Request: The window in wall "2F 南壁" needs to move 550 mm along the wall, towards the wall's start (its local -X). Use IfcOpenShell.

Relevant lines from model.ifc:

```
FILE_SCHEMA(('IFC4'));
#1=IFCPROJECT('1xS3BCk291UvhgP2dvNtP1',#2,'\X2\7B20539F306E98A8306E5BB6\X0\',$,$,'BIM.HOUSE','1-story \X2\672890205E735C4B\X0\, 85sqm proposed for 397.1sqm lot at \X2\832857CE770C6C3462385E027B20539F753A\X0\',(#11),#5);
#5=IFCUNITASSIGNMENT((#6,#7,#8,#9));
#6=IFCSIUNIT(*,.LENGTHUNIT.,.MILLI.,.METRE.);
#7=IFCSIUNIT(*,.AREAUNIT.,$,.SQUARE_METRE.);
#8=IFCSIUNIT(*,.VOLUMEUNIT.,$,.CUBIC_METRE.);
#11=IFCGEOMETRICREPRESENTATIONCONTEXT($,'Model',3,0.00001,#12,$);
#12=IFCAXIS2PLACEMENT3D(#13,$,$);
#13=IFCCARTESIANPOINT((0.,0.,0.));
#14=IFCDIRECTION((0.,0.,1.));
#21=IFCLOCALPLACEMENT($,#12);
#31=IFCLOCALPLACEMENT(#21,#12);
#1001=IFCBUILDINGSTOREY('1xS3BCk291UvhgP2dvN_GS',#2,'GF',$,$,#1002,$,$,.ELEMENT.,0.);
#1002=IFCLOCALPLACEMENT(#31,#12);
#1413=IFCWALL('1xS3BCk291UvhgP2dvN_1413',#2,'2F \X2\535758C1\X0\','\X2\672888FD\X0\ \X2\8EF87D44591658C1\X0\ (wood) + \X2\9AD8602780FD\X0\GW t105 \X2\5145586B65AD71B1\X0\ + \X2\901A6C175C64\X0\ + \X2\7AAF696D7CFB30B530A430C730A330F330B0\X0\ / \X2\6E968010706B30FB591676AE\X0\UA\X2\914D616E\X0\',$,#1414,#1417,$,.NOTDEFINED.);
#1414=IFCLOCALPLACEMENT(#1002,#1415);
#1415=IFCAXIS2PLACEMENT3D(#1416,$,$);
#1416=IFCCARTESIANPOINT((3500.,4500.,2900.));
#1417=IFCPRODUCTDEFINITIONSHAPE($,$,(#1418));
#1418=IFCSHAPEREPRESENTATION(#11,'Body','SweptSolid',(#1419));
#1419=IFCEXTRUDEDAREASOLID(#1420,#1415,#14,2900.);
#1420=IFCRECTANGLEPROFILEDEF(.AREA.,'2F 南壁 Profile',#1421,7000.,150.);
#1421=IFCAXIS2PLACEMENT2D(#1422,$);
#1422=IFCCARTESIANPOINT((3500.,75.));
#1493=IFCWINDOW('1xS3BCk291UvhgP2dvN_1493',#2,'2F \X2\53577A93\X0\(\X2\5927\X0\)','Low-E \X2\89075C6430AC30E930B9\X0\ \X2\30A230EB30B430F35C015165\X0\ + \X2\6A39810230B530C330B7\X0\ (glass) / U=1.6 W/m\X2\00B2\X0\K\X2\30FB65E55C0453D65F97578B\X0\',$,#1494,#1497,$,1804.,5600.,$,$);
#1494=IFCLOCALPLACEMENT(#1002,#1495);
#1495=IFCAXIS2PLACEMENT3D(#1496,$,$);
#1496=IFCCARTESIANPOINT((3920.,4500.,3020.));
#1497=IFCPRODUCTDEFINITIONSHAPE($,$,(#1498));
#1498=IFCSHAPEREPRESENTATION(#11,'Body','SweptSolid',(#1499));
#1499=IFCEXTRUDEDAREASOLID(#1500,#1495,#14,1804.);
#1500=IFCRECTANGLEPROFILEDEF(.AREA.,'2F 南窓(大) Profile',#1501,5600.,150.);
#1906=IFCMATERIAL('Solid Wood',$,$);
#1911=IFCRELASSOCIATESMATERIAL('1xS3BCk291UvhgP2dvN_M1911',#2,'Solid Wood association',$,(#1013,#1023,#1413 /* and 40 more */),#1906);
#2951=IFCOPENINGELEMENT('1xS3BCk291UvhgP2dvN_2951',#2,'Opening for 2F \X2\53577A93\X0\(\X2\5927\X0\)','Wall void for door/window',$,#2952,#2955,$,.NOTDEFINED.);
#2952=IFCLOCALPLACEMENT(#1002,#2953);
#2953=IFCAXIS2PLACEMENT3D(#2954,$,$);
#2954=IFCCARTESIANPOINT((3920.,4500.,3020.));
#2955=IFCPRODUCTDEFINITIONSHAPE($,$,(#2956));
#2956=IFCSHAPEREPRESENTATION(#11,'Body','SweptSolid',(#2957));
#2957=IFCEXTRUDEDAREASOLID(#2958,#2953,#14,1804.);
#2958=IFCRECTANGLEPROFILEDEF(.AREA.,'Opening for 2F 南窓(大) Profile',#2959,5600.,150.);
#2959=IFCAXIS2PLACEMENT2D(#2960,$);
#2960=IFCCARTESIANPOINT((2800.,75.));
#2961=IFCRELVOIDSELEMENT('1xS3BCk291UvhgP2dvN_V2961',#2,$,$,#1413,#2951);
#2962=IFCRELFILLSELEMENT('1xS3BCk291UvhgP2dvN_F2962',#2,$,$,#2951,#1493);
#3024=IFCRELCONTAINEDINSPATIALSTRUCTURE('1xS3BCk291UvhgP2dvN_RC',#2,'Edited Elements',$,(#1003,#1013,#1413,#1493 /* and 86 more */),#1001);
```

```python
import ifcopenshell
import ifcopenshell.api.geometry
import ifcopenshell.util.placement

model = ifcopenshell.open("model.ifc")

window = model.by_guid("1xS3BCk291UvhgP2dvN_1493")
opening = window.FillsVoids[0].RelatingOpeningElement
wall = opening.VoidsElements[0].RelatingBuildingElement

wall_matrix = ifcopenshell.util.placement.get_local_placement(wall.ObjectPlacement)
shift = wall_matrix[:3, 0] * -550.0
before = ifcopenshell.util.placement.get_local_placement(window.ObjectPlacement)[:3, 3].copy()

# The window is not placed relative to its opening, so move both.
for product in (opening, window):
    matrix = ifcopenshell.util.placement.get_local_placement(product.ObjectPlacement)
    matrix[:3, 3] += shift
    ifcopenshell.api.geometry.edit_object_placement(model, product=product, matrix=matrix, is_si=False)

after = ifcopenshell.util.placement.get_local_placement(window.ObjectPlacement)[:3, 3]
print("window moved by", (after - before).round(3) + 0.0)

model.write("model_v2.ifc")
```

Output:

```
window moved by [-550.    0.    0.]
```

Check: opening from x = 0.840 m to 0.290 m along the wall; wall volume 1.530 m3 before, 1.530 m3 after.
